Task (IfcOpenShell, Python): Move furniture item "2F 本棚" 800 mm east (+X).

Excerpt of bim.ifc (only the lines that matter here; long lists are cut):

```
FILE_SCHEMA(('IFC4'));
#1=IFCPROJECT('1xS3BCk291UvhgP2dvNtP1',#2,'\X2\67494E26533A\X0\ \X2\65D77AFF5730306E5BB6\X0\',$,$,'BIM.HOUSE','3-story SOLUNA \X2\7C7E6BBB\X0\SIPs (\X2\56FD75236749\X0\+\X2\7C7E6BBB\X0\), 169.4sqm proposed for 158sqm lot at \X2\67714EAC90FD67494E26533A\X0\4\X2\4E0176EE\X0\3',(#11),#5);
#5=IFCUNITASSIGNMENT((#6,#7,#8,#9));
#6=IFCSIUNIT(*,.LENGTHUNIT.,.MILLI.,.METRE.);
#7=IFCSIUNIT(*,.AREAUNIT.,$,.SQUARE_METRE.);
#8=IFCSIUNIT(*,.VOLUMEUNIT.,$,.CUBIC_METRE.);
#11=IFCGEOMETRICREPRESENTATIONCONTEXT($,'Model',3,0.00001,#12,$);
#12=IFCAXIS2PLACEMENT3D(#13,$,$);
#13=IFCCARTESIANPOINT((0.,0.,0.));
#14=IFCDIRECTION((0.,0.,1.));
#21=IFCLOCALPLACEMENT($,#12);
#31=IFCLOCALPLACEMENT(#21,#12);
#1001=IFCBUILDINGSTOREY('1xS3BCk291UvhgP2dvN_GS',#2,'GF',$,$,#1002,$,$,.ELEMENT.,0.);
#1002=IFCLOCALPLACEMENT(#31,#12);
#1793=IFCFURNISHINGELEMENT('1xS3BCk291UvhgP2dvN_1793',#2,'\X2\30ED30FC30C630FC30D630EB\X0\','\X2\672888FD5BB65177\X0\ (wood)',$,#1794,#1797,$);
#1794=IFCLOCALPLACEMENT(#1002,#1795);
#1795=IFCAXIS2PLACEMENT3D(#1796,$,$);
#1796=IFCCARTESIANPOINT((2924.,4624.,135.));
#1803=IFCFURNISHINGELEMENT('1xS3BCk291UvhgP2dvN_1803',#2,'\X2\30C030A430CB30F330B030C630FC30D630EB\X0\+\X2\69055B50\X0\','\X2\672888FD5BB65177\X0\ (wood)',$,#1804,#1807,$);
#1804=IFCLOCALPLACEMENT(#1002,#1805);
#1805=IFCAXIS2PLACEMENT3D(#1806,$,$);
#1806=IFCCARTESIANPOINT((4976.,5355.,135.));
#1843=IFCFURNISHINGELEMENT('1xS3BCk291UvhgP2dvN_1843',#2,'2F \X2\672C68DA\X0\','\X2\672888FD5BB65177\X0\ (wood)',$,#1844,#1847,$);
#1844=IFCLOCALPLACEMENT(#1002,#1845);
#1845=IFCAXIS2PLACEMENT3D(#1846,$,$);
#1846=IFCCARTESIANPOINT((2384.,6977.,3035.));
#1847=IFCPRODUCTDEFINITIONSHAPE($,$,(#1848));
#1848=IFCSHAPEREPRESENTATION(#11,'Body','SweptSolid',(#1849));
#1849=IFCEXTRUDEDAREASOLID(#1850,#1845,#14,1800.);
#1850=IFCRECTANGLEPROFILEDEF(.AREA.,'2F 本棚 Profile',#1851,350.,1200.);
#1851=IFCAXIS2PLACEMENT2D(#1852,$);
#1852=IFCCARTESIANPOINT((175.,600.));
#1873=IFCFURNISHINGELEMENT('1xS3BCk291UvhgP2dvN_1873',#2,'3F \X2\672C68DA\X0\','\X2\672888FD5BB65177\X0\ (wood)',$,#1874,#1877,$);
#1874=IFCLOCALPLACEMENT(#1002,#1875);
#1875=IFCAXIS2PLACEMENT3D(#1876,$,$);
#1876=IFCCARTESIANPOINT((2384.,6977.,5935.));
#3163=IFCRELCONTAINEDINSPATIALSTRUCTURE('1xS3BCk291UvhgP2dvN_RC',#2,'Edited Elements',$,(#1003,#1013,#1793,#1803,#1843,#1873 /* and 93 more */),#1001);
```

```python
import ifcopenshell
import ifcopenshell.api.geometry
import ifcopenshell.util.placement
import ifcopenshell.util.unit

model = ifcopenshell.open("bim.ifc")
unit_scale = ifcopenshell.util.unit.calculate_unit_scale(model)

item = model.by_id(1843)
matrix = ifcopenshell.util.placement.get_local_placement(item.ObjectPlacement)
matrix[0, 3] += 0.8 / unit_scale
ifcopenshell.api.geometry.edit_object_placement(model, product=item, matrix=matrix, is_si=False)

print(ifcopenshell.util.placement.get_local_placement(item.ObjectPlacement).round(3) + 0.0)

model.write("bim-out.ifc")
```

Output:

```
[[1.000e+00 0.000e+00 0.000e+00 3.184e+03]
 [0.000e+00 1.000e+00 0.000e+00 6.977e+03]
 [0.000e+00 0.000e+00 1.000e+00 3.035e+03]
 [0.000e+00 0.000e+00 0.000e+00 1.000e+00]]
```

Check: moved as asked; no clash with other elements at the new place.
